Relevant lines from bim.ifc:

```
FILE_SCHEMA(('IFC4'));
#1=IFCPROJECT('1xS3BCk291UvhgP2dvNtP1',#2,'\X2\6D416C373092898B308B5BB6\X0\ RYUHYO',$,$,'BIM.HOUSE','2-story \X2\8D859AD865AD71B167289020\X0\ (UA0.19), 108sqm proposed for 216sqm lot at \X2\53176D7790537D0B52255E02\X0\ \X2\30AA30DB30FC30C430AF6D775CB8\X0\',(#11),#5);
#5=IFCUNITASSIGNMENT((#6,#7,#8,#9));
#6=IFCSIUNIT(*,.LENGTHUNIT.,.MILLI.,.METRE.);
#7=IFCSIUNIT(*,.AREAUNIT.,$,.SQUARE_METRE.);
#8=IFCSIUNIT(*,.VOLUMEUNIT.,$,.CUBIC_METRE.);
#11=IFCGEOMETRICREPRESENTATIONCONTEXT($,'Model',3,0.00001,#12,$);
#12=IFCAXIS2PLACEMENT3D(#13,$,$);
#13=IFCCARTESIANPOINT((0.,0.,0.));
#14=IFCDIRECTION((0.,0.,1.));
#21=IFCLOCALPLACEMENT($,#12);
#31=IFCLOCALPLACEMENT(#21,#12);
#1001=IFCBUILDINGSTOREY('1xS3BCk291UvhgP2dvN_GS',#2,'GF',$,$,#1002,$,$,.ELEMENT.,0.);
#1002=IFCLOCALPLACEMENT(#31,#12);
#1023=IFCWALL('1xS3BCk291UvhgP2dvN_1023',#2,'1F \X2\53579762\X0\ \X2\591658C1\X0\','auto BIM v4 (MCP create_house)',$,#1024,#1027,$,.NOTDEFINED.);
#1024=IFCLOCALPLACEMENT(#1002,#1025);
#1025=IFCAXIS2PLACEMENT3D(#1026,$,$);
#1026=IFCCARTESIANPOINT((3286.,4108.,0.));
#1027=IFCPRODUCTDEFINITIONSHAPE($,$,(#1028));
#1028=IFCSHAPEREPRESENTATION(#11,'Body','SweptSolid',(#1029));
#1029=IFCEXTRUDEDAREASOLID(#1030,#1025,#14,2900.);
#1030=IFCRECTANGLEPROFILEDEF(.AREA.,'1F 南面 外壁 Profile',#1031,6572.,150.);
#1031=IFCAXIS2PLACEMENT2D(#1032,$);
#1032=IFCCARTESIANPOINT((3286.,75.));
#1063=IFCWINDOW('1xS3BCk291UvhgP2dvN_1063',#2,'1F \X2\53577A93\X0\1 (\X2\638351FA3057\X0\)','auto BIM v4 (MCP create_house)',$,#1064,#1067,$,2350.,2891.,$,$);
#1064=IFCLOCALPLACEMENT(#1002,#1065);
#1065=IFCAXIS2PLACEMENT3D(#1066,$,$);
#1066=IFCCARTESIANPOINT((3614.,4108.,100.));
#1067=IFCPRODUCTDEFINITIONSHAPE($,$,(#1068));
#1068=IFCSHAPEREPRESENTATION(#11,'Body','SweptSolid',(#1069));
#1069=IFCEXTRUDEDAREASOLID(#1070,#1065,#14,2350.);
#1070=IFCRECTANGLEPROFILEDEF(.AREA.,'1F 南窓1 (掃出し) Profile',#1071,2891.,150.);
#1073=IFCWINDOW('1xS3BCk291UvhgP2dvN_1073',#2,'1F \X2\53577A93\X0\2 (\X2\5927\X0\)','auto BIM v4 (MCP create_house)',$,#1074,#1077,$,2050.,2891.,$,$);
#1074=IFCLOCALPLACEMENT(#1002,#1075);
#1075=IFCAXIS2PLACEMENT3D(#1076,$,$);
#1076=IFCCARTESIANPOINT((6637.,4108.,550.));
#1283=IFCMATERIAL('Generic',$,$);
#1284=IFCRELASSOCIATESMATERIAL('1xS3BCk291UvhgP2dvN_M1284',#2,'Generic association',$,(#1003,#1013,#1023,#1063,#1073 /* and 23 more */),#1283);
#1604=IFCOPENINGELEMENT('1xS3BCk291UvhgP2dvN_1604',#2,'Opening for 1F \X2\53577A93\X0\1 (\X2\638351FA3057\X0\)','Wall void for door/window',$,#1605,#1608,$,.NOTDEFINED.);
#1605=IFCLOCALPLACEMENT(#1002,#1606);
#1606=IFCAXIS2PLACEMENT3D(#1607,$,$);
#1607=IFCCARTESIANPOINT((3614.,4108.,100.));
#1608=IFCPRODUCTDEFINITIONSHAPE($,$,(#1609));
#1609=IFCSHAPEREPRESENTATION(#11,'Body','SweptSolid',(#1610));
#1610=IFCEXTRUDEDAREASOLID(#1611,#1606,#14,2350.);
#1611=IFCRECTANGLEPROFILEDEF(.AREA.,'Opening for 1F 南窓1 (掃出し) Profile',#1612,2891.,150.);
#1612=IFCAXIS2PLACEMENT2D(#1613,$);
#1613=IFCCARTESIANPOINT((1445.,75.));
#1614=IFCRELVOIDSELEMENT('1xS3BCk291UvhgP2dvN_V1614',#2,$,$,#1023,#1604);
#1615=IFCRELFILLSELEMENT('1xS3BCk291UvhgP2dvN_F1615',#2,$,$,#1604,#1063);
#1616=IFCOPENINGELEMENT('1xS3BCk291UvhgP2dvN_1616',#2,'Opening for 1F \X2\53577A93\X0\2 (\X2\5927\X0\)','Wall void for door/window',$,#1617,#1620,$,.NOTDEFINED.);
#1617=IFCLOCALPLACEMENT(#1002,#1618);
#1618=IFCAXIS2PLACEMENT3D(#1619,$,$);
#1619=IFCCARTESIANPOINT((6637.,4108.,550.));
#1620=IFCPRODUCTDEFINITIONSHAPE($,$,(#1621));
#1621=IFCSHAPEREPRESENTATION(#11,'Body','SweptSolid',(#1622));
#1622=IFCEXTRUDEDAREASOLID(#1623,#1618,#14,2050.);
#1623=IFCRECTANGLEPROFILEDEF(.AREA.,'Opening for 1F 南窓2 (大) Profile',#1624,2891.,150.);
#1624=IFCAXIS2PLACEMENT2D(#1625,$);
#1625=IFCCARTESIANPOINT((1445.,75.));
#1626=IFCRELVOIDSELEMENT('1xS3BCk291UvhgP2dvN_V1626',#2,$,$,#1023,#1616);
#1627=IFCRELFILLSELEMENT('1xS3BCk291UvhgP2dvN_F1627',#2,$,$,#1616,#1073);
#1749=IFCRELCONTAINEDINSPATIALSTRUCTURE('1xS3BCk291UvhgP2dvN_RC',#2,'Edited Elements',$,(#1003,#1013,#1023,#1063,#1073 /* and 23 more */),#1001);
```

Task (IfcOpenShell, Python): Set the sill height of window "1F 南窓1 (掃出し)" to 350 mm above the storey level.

```python
import numpy as np
import ifcopenshell
import ifcopenshell.api.geometry
import ifcopenshell.geom
import ifcopenshell.util.element
import ifcopenshell.util.placement
import ifcopenshell.util.shape
import ifcopenshell.util.unit

model = ifcopenshell.open("bim.ifc")
unit_scale = ifcopenshell.util.unit.calculate_unit_scale(model)

window = model.by_guid("1xS3BCk291UvhgP2dvN_1063")
opening = window.FillsVoids[0].RelatingOpeningElement
storey = ifcopenshell.util.element.get_container(window, ifc_class="IfcBuildingStorey")
level = ifcopenshell.util.placement.get_local_placement(storey.ObjectPlacement)[2, 3]

# The opening's origin need not be at the sill, so measure its lowest point.
shape = ifcopenshell.geom.create_shape(ifcopenshell.geom.settings(), opening)
bottom = ifcopenshell.util.shape.get_shape_bottom_elevation(shape, shape.geometry) / unit_scale
dz = level + 350.0 - bottom

shift = np.array([0.0, 0.0, dz])
# The window is not placed relative to its opening, so move both.
for product in (opening, window):
    matrix = ifcopenshell.util.placement.get_local_placement(product.ObjectPlacement)
    matrix[:3, 3] += shift
    ifcopenshell.api.geometry.edit_object_placement(model, product=product, matrix=matrix, is_si=False)

print(f"moved by {dz * unit_scale:+.3f} m")

model.write("bim_updated.ifc")
```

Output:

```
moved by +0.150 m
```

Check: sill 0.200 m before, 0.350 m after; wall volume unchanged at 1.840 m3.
